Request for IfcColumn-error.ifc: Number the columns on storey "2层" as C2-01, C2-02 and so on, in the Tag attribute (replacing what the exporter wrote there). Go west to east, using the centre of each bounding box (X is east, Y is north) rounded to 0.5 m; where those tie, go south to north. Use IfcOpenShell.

First a look at what the model holds.

```python
import ifcopenshell
import ifcopenshell.util.element
import ifcopenshell.util.placement

model = ifcopenshell.open("IfcColumn-error.ifc")
print(model.schema)
storey = next(s for s in model.by_type("IfcBuildingStorey") if s.Name == "2层")
columns = [e for e in ifcopenshell.util.element.get_decomposition(storey) if e.is_a("IfcColumn")]
for e in sorted(columns, key=lambda e: e.id()):
    origin = ifcopenshell.util.placement.get_local_placement(e.ObjectPlacement)[:3, 3]
    print(e.id(), e.Tag, e.Name, origin.round(2) + 0.0, sep=" | ")
```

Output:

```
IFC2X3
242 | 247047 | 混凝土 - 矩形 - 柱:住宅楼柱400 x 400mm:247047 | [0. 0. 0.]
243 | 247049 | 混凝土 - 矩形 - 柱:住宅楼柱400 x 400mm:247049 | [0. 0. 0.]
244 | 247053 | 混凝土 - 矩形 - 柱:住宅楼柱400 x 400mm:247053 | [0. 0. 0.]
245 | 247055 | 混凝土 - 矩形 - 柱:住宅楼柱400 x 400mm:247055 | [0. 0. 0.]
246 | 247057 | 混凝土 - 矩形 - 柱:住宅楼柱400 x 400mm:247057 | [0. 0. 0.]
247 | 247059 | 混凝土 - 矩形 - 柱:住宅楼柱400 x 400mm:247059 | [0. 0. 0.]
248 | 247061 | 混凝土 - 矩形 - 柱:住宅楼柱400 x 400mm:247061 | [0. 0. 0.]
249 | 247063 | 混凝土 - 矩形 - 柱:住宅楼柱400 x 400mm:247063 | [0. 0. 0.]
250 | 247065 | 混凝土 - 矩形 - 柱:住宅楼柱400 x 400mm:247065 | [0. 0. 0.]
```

```python
import ifcopenshell
import ifcopenshell.geom
import ifcopenshell.util.element
import ifcopenshell.util.shape

model = ifcopenshell.open("IfcColumn-error.ifc")
settings = ifcopenshell.geom.settings()
settings.set("use-world-coords", True)


def centre(element):
    shape = ifcopenshell.geom.create_shape(settings, element)
    return ifcopenshell.util.shape.get_bbox_centroid(shape.geometry)


storey = next(s for s in model.by_type("IfcBuildingStorey") if s.Name == "2层")
columns = [e for e in ifcopenshell.util.element.get_decomposition(storey) if e.is_a("IfcColumn")]

# Insertion points can sit at a corner or the storey origin, so sort by the geometry (in metres).
centres = {e: centre(e) for e in columns}
columns.sort(key=lambda e: (round(centres[e][0] / 0.5), centres[e][1]))

for i, e in enumerate(columns, start=1):
    number = f"C2-{i:02d}"
    e.Tag = number
    print(e.id(), number)

model.write("IfcColumn-error-out.ifc")
```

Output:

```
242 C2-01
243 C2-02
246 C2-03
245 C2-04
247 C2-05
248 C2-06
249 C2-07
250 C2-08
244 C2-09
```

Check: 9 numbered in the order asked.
